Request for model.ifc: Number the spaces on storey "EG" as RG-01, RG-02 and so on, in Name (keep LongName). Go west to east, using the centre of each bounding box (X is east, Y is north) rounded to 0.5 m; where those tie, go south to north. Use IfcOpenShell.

First a look at what the model holds.

```python
import ifcopenshell
import ifcopenshell.util.element
import ifcopenshell.util.placement

model = ifcopenshell.open("model.ifc")
print(model.schema)
storey = next(s for s in model.by_type("IfcBuildingStorey") if s.Name == "EG")
spaces = [e for e in ifcopenshell.util.element.get_decomposition(storey) if e.is_a("IfcSpace")]
for e in sorted(spaces, key=lambda e: e.id()):
    origin = ifcopenshell.util.placement.get_local_placement(e.ObjectPlacement)[:3, 3]
    print(e.id(), e.Name, e.LongName, origin.round(2) + 0.0, sep=" | ")
```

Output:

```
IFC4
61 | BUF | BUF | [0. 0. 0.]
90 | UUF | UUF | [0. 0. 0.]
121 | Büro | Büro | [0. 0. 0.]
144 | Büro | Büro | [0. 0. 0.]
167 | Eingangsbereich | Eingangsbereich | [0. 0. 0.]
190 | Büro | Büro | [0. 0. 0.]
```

```python
import ifcopenshell
import ifcopenshell.geom
import ifcopenshell.util.element
import ifcopenshell.util.shape

model = ifcopenshell.open("model.ifc")
settings = ifcopenshell.geom.settings()
settings.set("use-world-coords", True)


def centre(element):
    shape = ifcopenshell.geom.create_shape(settings, element)
    return ifcopenshell.util.shape.get_bbox_centroid(shape.geometry)


storey = next(s for s in model.by_type("IfcBuildingStorey") if s.Name == "EG")
spaces = [e for e in ifcopenshell.util.element.get_decomposition(storey) if e.is_a("IfcSpace")]

# Insertion points can sit at a corner or the storey origin, so sort by the geometry (in metres).
centres = {e: centre(e) for e in spaces}
spaces.sort(key=lambda e: (round(centres[e][0] / 0.5), centres[e][1]))

for i, e in enumerate(spaces, start=1):
    number = f"RG-{i:02d}"
    e.Name = number
    print(e.id(), number)

model.write("model_edited.ifc")
```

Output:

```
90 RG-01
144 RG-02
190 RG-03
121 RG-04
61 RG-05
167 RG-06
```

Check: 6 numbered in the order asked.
